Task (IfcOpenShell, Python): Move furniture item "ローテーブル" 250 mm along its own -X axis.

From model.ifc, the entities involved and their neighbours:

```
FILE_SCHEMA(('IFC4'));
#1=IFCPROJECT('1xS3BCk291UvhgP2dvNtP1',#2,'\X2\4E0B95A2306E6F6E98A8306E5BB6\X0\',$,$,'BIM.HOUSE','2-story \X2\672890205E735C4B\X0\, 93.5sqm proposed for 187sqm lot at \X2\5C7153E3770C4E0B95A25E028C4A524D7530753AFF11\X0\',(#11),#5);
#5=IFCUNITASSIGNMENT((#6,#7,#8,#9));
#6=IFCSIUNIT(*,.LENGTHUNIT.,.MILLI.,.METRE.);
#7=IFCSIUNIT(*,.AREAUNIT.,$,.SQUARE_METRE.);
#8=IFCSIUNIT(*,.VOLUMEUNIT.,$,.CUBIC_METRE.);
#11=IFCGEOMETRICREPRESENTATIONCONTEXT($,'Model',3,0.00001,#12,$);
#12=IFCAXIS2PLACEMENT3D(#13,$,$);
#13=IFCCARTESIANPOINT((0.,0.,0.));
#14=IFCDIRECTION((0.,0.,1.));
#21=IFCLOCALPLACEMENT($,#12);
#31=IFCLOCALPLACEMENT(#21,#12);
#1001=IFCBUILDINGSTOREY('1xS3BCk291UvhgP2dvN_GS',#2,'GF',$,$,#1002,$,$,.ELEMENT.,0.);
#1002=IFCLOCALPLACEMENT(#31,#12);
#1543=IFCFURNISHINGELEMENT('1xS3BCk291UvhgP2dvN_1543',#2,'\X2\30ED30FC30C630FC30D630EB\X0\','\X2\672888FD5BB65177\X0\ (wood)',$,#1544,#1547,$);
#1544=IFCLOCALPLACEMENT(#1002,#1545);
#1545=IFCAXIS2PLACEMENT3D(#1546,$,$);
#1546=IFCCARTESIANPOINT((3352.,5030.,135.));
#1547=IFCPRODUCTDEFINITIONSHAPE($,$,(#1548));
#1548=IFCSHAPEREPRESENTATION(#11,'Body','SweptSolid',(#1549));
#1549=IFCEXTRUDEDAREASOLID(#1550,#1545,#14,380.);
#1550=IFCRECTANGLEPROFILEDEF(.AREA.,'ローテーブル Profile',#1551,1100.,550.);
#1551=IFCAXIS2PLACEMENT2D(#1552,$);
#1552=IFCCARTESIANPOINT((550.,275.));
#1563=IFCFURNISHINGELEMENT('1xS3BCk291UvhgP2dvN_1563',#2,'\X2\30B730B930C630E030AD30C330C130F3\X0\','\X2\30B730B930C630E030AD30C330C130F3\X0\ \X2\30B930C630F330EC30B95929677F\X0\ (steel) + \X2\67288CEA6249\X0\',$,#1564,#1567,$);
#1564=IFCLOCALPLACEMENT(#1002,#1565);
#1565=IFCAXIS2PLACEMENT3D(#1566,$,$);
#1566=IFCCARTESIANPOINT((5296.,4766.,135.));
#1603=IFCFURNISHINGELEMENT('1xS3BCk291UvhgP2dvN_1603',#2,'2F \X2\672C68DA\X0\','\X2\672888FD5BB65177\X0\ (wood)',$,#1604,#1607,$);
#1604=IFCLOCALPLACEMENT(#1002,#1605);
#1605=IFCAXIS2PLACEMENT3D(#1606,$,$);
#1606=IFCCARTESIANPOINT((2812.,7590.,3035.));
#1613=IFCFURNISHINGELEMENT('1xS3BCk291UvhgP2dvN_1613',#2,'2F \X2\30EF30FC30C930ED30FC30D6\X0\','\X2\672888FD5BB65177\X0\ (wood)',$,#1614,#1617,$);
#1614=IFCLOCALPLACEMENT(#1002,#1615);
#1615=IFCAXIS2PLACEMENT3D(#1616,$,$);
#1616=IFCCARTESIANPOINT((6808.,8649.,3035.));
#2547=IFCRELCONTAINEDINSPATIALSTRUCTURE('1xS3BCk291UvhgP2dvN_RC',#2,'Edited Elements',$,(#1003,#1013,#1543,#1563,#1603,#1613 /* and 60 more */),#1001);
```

```python
import ifcopenshell
import ifcopenshell.api.geometry
import ifcopenshell.util.placement
import ifcopenshell.util.unit

model = ifcopenshell.open("model.ifc")
unit_scale = ifcopenshell.util.unit.calculate_unit_scale(model)

item = model.by_guid("1xS3BCk291UvhgP2dvN_1543")
matrix = ifcopenshell.util.placement.get_local_placement(item.ObjectPlacement)
matrix[:3, 3] -= matrix[:3, 0] * 0.25 / unit_scale
ifcopenshell.api.geometry.edit_object_placement(model, product=item, matrix=matrix, is_si=False)

print(ifcopenshell.util.placement.get_local_placement(item.ObjectPlacement).round(3) + 0.0)

model.write("model_v2.ifc")
```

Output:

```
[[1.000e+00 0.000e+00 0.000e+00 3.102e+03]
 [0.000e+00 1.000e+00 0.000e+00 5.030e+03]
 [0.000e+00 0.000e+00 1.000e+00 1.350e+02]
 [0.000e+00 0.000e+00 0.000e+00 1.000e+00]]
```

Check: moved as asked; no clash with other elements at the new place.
